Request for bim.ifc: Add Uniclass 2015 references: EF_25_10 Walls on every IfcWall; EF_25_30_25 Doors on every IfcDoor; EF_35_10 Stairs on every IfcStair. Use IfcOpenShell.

First a look at what the model holds.

```python
import ifcopenshell

model = ifcopenshell.open("bim.ifc")
print(model.schema)
print("classifications:", [c.Name for c in model.by_type("IfcClassification")])
for ifc_class in ("IfcDoor", "IfcRoof", "IfcStair", "IfcWall", "IfcWindow"):
    print(ifc_class, len(model.by_type(ifc_class)))
```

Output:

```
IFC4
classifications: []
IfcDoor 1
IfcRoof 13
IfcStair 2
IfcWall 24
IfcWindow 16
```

```python
import ifcopenshell
import ifcopenshell.api.classification

model = ifcopenshell.open("bim.ifc")

system = ifcopenshell.api.classification.add_classification(model, classification="Uniclass 2015")

codes = {
    "IfcWall": ("EF_25_10", "Walls"),
    "IfcDoor": ("EF_25_30_25", "Doors"),
    "IfcStair": ("EF_35_10", "Stairs"),
}
for ifc_class, (code, name) in codes.items():
    products = model.by_type(ifc_class)
    ifcopenshell.api.classification.add_reference(
        model, products=products, classification=system, identification=code, name=name
    )
    print(code, len(products))

model.write("bim_updated.ifc")
```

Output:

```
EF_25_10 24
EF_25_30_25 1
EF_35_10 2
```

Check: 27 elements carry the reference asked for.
